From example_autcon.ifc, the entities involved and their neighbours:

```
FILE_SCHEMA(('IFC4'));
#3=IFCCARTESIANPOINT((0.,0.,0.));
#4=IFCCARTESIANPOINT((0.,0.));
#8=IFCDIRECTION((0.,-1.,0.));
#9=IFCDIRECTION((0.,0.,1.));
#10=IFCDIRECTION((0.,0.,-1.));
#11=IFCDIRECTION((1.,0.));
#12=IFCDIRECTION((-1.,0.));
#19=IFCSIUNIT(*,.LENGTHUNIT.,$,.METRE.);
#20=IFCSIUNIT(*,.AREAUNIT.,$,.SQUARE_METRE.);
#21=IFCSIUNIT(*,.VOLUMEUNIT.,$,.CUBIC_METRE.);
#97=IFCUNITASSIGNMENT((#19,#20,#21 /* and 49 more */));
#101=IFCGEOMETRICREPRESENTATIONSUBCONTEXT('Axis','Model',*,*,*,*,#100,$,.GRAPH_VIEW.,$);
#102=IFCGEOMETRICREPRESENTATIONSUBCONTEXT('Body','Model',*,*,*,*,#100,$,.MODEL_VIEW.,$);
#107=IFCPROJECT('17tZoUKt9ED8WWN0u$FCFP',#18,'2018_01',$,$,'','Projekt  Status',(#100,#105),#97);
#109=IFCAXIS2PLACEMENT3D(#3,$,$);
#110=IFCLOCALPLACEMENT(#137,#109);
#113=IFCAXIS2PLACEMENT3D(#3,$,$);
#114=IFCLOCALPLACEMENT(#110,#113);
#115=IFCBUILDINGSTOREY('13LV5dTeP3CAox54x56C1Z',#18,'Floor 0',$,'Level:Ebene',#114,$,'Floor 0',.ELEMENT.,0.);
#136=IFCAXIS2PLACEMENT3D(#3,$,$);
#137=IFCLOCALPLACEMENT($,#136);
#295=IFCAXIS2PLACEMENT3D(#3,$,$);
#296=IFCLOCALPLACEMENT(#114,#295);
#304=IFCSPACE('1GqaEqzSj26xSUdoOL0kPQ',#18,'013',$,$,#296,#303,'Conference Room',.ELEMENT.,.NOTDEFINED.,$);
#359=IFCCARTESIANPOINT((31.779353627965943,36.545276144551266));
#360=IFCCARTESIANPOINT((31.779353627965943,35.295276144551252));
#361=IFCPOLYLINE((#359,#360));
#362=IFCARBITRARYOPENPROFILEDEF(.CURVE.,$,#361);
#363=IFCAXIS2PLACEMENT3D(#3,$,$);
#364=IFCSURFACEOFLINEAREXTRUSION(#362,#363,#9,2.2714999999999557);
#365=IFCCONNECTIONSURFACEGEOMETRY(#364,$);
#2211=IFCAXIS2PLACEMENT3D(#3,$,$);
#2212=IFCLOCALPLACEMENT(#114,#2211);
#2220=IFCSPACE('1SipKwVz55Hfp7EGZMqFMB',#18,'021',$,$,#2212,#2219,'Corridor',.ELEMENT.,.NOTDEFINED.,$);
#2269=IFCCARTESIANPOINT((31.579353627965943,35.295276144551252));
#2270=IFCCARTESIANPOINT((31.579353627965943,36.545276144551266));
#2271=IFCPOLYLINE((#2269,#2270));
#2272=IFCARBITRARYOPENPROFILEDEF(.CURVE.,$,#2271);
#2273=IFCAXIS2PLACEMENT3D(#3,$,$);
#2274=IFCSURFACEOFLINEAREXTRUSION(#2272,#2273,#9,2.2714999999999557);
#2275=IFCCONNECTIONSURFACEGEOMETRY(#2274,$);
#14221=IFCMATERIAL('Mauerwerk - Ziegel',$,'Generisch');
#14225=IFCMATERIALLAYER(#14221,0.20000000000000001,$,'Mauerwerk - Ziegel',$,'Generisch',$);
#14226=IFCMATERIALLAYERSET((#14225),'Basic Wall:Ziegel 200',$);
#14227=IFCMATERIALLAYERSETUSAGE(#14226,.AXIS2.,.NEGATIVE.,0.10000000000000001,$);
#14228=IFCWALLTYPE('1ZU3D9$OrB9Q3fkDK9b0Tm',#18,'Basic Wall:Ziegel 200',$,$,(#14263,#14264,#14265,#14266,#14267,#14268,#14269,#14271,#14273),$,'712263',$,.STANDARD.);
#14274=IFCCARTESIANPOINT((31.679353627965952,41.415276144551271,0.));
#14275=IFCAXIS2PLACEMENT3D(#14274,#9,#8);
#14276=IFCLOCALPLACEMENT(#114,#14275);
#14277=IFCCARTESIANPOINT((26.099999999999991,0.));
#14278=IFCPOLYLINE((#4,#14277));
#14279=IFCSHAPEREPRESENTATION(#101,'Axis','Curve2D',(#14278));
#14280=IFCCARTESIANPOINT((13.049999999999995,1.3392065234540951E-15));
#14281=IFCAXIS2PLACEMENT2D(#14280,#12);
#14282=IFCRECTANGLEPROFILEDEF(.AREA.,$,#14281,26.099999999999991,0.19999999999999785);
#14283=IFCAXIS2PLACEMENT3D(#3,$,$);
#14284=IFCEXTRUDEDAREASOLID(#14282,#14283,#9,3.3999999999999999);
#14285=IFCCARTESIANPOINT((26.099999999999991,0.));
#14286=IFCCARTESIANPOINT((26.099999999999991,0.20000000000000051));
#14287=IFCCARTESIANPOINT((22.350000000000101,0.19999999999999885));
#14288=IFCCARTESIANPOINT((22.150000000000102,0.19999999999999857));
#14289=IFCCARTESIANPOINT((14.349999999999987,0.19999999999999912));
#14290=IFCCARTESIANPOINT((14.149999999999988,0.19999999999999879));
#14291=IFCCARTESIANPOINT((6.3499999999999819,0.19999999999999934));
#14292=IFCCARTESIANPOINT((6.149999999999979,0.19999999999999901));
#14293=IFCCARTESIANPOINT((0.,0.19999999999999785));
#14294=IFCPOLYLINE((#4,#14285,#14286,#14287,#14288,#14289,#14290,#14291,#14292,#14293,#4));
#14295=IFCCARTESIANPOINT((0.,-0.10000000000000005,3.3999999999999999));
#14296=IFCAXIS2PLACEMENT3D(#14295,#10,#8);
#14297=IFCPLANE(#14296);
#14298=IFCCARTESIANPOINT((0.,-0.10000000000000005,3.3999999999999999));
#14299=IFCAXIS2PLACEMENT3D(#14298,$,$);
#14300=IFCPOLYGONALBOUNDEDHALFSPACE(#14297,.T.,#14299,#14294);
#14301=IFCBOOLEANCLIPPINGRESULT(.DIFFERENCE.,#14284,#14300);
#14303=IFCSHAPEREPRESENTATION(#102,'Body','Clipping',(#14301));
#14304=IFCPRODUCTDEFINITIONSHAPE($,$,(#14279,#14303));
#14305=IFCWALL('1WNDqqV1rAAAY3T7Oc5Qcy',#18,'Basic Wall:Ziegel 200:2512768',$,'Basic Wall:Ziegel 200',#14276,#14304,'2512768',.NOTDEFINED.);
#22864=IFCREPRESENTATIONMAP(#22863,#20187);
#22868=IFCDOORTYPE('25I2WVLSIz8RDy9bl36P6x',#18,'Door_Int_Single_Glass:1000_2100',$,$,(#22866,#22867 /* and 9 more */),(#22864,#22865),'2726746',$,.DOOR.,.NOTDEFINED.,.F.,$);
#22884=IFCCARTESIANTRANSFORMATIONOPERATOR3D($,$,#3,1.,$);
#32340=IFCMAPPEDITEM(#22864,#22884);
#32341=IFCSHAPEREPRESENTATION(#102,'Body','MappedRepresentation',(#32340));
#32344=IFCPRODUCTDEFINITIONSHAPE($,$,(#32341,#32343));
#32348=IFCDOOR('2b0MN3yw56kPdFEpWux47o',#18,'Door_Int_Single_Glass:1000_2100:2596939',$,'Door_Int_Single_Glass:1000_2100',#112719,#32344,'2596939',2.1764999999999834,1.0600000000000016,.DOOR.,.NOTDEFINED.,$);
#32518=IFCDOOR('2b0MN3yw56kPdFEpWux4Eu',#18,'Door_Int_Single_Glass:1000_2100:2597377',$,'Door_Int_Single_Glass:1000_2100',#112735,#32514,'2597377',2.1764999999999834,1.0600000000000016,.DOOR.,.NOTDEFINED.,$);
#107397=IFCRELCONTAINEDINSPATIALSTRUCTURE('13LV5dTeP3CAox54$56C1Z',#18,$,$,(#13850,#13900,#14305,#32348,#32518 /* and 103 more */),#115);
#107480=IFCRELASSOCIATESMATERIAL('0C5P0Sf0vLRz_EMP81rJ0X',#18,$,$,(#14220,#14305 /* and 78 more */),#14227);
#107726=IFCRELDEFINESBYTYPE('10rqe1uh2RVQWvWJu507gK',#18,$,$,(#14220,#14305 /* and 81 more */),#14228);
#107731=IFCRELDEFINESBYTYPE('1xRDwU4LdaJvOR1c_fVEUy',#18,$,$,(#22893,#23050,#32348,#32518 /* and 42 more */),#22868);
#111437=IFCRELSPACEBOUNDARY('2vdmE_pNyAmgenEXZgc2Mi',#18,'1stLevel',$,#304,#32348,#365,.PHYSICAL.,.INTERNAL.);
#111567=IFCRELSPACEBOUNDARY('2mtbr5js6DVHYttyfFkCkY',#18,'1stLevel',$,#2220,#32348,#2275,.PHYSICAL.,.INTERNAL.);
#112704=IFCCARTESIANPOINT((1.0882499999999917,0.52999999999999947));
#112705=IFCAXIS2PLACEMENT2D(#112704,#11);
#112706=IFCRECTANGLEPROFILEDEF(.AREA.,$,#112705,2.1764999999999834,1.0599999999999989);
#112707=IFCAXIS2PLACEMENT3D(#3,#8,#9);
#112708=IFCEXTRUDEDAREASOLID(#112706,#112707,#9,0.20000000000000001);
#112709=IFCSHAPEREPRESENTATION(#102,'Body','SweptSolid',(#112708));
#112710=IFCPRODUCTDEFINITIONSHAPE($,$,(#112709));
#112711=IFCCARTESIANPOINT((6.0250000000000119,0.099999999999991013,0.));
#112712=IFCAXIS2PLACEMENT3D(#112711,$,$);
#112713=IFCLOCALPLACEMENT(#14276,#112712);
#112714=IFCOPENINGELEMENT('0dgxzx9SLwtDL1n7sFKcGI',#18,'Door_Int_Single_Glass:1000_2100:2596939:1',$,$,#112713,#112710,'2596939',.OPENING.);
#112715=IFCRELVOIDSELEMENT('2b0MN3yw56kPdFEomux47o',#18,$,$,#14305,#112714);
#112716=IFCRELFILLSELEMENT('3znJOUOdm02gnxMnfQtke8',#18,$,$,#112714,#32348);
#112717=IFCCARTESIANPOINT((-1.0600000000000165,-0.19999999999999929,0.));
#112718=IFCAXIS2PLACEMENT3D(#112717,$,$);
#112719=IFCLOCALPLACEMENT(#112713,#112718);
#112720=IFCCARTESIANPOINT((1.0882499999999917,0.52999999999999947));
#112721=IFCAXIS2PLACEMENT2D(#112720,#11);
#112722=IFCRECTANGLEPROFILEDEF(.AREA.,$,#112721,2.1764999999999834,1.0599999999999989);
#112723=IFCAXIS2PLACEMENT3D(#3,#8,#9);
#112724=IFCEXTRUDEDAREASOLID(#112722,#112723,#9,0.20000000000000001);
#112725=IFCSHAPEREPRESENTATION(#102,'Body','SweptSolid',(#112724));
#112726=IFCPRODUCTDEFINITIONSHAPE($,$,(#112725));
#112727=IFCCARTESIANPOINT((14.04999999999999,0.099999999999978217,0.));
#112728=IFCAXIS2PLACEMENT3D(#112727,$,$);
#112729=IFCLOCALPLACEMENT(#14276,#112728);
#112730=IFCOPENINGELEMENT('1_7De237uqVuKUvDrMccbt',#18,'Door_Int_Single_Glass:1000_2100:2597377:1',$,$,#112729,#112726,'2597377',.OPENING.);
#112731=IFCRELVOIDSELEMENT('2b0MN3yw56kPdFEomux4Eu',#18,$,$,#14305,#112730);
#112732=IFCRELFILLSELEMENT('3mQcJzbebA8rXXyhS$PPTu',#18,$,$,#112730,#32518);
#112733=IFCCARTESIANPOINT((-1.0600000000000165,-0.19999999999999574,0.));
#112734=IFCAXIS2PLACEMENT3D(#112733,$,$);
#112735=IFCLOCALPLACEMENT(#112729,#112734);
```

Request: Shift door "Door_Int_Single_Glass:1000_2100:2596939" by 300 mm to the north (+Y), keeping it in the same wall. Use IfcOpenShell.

```python
import numpy as np
import ifcopenshell
import ifcopenshell.api.geometry
import ifcopenshell.util.placement

model = ifcopenshell.open("example_autcon.ifc")

door = model.by_id(32348)
opening = door.FillsVoids[0].RelatingOpeningElement
wall = opening.VoidsElements[0].RelatingBuildingElement

wall_matrix = ifcopenshell.util.placement.get_local_placement(wall.ObjectPlacement)
shift = wall_matrix[:3, 0] * -0.3
before = ifcopenshell.util.placement.get_local_placement(door.ObjectPlacement)[:3, 3].copy()

# The door is placed relative to its opening, so it follows when the opening moves.
matrix = ifcopenshell.util.placement.get_local_placement(opening.ObjectPlacement)
matrix[:3, 3] += shift
ifcopenshell.api.geometry.edit_object_placement(
    model, product=opening, matrix=matrix, is_si=False, should_transform_children=True
)

# Space boundary surfaces are stored in each space's coordinates; move them too.
for rel in door.ProvidesBoundaries:
    if not rel.ConnectionGeometry:
        continue
    surface = rel.ConnectionGeometry.SurfaceOnRelatingElement
    space_matrix = ifcopenshell.util.placement.get_local_placement(rel.RelatingSpace.ObjectPlacement)
    point = np.array(surface.Position.Location.Coordinates) + space_matrix[:3, :3].T @ shift
    surface.Position = model.createIfcAxis2Placement3D(
        model.createIfcCartesianPoint(point.tolist()), surface.Position.Axis, surface.Position.RefDirection
    )

after = ifcopenshell.util.placement.get_local_placement(door.ObjectPlacement)[:3, 3]
print("door moved by", (after - before).round(3) + 0.0)

model.write("example_autcon_v2.ifc")
```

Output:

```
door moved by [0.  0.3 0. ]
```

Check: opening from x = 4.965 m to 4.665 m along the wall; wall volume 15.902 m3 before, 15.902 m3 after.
